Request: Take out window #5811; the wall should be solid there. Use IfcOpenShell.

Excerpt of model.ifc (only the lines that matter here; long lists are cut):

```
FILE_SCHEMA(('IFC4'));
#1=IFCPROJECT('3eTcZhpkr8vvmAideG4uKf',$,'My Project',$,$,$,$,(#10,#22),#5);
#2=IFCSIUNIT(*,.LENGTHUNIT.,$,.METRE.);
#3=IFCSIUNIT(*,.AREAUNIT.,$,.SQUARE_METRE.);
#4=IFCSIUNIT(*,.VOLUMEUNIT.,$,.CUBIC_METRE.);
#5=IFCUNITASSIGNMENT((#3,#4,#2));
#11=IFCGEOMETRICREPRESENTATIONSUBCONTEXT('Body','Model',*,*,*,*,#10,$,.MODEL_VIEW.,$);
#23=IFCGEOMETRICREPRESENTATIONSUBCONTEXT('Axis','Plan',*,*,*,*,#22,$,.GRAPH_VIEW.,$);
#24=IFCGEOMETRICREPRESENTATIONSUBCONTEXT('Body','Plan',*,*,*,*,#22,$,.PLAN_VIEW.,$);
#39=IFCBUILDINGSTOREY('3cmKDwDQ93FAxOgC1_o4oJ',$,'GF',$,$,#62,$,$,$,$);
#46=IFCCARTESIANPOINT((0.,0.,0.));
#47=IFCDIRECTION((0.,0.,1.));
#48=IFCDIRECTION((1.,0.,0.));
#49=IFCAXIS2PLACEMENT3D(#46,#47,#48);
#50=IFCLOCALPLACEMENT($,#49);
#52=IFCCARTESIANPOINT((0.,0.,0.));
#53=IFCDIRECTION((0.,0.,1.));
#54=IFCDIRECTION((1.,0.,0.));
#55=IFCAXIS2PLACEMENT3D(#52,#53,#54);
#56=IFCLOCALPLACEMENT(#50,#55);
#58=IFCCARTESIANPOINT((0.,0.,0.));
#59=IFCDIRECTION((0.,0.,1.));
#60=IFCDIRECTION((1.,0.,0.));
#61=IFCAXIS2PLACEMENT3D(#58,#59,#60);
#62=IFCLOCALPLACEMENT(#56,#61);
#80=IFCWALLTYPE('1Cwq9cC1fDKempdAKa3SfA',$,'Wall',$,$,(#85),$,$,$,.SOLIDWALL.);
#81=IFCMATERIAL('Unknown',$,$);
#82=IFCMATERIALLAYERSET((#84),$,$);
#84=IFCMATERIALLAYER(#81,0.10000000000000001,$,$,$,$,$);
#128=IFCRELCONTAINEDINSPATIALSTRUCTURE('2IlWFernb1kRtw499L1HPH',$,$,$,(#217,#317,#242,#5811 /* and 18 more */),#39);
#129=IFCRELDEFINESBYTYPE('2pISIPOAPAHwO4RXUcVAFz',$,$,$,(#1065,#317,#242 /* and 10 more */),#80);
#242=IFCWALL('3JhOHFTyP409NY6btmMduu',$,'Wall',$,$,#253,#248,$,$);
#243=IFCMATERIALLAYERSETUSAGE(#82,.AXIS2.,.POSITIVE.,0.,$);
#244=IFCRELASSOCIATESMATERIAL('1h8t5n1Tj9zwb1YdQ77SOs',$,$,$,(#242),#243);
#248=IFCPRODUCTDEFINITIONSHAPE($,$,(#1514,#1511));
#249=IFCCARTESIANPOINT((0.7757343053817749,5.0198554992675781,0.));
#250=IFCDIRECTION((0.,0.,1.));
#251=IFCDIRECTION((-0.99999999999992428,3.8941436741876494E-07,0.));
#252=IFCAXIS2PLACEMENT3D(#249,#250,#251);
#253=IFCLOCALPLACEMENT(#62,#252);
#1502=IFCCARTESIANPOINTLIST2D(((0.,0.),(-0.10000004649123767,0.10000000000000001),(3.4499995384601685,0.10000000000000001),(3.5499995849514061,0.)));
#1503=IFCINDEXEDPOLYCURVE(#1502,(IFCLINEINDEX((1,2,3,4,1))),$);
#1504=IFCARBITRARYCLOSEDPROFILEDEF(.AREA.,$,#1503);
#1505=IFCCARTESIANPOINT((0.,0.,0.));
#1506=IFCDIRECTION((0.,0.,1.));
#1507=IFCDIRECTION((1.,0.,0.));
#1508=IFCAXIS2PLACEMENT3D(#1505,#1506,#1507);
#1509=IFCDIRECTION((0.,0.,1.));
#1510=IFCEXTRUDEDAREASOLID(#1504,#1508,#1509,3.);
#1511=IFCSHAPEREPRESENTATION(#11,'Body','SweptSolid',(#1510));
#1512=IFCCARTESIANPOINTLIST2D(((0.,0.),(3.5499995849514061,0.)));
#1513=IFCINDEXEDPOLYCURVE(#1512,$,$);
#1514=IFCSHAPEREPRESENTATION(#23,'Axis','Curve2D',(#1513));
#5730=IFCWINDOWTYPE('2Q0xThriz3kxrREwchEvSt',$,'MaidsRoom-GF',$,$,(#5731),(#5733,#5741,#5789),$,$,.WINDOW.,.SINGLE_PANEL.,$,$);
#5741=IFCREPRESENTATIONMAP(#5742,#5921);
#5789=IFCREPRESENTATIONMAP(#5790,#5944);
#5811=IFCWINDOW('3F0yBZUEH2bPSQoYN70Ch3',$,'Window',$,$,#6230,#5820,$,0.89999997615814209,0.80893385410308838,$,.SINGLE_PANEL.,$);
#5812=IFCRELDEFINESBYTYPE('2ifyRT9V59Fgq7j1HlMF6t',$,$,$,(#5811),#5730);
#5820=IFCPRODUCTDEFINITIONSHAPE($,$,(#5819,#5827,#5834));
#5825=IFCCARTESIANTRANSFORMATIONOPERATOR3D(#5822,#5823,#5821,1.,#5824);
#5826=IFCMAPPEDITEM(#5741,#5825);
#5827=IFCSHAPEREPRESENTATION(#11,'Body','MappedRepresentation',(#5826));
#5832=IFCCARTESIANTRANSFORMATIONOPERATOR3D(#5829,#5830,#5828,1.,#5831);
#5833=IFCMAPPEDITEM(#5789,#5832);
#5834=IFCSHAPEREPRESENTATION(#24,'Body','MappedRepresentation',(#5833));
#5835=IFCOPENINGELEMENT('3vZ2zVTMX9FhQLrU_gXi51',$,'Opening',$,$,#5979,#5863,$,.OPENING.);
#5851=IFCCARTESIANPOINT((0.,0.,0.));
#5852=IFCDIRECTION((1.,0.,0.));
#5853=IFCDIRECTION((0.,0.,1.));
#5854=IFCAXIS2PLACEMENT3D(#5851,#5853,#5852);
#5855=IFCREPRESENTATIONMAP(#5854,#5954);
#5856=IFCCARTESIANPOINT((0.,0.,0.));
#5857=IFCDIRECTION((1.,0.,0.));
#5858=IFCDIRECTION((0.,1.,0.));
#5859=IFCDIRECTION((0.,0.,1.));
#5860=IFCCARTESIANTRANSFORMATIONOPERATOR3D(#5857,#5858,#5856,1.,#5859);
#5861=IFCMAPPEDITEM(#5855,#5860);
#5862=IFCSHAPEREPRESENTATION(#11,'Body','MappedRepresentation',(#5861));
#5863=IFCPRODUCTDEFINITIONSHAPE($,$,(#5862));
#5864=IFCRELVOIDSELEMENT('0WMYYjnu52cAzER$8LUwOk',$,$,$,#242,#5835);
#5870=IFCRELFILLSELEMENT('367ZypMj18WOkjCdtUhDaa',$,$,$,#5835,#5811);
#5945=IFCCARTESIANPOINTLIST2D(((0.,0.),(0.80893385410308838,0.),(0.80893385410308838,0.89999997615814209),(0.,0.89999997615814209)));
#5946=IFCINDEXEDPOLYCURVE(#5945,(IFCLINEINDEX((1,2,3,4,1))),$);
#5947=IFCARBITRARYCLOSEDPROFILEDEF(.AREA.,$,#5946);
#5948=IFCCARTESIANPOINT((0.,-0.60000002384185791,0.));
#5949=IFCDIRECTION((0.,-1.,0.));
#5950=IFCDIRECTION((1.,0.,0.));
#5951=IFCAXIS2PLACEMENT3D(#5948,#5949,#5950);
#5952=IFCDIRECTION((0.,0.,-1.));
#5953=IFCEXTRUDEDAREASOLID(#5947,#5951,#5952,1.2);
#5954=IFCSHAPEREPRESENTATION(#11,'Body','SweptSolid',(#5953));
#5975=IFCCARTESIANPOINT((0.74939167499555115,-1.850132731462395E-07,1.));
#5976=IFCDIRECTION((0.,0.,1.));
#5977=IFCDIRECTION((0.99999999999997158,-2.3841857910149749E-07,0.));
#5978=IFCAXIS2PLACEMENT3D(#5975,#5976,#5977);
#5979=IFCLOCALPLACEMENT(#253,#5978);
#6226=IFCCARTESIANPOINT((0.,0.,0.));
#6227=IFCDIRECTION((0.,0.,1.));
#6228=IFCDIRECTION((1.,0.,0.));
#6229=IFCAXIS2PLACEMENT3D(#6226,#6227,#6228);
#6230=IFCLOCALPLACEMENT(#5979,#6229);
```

```python
import ifcopenshell
import ifcopenshell.api.feature
import ifcopenshell.api.root
import ifcopenshell.geom
import ifcopenshell.util.shape

model = ifcopenshell.open("model.ifc")
settings = ifcopenshell.geom.settings()


def volume(element):
    """Net volume in cubic metres, openings subtracted."""
    shape = ifcopenshell.geom.create_shape(settings, element)
    return ifcopenshell.util.shape.get_volume(shape.geometry)


window = model.by_guid("3F0yBZUEH2bPSQoYN70Ch3")
opening = window.FillsVoids[0].RelatingOpeningElement
wall = opening.VoidsElements[0].RelatingBuildingElement
before = volume(wall)

ifcopenshell.api.root.remove_product(model, product=window)
ifcopenshell.api.feature.remove_feature(model, feature=opening)

after = volume(wall)

print(f"wall volume {before:.3f} -> {after:.3f} m3")

model.write("model_rev.ifc")
```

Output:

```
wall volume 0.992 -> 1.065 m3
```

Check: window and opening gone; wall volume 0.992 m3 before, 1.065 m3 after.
